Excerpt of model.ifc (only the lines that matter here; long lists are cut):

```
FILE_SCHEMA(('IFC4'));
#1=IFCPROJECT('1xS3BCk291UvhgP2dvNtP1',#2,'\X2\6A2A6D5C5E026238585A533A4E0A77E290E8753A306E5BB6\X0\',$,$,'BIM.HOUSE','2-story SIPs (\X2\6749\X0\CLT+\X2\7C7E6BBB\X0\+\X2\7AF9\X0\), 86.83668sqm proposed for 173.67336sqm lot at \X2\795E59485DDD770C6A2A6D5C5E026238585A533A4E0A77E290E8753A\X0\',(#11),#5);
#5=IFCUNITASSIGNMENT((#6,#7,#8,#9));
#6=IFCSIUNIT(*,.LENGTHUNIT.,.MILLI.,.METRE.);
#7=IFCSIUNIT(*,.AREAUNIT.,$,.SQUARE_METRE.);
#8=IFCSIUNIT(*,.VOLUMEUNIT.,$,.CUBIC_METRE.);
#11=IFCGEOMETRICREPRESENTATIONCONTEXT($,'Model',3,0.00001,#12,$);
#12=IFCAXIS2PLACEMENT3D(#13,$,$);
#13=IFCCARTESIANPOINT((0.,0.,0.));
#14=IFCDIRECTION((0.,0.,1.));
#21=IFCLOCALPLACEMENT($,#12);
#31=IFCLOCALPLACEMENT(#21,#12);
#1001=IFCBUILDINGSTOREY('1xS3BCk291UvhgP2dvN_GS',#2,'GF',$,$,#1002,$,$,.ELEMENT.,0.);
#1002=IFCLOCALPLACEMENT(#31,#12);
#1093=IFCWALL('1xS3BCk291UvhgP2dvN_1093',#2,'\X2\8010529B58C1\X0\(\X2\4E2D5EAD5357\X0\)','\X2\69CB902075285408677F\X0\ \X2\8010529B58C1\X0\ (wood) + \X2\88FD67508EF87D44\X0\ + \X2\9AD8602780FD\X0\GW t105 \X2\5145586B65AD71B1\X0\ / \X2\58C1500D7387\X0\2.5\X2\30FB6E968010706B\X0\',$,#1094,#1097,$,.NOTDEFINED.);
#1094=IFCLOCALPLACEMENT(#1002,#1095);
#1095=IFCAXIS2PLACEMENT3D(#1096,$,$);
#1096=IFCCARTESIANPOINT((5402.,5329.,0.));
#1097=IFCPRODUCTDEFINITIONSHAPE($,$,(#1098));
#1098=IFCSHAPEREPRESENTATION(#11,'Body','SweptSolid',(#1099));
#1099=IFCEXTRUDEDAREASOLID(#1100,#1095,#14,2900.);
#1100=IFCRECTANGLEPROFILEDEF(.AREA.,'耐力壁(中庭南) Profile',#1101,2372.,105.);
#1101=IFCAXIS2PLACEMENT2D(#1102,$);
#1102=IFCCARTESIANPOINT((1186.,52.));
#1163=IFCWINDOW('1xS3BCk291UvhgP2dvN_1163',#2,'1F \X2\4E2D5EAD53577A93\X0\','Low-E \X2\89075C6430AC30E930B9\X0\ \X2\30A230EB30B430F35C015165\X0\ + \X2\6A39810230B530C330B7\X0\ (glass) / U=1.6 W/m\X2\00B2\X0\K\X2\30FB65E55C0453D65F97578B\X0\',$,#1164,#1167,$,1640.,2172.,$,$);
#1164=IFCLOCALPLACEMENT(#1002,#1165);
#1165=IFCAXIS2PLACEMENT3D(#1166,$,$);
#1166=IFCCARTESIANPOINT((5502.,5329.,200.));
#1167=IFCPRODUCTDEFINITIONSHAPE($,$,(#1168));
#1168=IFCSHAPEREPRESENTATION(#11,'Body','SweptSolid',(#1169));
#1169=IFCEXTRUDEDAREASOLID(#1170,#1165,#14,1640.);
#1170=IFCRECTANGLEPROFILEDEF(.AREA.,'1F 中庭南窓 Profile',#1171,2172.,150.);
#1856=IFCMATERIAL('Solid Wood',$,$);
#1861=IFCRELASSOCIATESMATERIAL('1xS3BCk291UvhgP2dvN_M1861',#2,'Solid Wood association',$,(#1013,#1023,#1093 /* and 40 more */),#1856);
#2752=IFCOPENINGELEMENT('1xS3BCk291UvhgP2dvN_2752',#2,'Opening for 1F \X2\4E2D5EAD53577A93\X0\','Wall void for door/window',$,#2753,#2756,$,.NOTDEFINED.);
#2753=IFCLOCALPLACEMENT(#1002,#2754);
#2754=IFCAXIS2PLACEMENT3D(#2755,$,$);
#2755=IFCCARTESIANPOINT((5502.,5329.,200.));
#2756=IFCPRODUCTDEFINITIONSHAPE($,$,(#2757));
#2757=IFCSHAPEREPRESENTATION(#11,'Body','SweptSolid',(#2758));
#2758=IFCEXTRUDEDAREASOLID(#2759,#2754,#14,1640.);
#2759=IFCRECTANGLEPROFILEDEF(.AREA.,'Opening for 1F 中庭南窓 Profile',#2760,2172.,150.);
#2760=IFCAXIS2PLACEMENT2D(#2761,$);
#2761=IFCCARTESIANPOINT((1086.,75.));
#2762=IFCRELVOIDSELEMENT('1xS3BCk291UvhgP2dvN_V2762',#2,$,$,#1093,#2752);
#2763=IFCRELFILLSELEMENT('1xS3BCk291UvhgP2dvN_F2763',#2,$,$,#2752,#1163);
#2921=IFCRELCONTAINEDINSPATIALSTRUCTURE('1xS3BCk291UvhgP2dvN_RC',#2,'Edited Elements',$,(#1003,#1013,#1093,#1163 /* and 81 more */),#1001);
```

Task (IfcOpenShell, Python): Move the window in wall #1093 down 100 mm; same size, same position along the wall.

```python
import numpy as np
import ifcopenshell
import ifcopenshell.api.geometry
import ifcopenshell.util.placement
import ifcopenshell.util.unit

model = ifcopenshell.open("model.ifc")
unit_scale = ifcopenshell.util.unit.calculate_unit_scale(model)

window = model.by_id(1163)
opening = window.FillsVoids[0].RelatingOpeningElement
dz = -0.1 / unit_scale

shift = np.array([0.0, 0.0, dz])
# The window is not placed relative to its opening, so move both.
for product in (opening, window):
    matrix = ifcopenshell.util.placement.get_local_placement(product.ObjectPlacement)
    matrix[:3, 3] += shift
    ifcopenshell.api.geometry.edit_object_placement(model, product=product, matrix=matrix, is_si=False)

print(f"moved by {dz * unit_scale:+.3f} m")

model.write("model_rev.ifc")
```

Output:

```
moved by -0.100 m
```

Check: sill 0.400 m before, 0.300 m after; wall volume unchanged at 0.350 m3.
